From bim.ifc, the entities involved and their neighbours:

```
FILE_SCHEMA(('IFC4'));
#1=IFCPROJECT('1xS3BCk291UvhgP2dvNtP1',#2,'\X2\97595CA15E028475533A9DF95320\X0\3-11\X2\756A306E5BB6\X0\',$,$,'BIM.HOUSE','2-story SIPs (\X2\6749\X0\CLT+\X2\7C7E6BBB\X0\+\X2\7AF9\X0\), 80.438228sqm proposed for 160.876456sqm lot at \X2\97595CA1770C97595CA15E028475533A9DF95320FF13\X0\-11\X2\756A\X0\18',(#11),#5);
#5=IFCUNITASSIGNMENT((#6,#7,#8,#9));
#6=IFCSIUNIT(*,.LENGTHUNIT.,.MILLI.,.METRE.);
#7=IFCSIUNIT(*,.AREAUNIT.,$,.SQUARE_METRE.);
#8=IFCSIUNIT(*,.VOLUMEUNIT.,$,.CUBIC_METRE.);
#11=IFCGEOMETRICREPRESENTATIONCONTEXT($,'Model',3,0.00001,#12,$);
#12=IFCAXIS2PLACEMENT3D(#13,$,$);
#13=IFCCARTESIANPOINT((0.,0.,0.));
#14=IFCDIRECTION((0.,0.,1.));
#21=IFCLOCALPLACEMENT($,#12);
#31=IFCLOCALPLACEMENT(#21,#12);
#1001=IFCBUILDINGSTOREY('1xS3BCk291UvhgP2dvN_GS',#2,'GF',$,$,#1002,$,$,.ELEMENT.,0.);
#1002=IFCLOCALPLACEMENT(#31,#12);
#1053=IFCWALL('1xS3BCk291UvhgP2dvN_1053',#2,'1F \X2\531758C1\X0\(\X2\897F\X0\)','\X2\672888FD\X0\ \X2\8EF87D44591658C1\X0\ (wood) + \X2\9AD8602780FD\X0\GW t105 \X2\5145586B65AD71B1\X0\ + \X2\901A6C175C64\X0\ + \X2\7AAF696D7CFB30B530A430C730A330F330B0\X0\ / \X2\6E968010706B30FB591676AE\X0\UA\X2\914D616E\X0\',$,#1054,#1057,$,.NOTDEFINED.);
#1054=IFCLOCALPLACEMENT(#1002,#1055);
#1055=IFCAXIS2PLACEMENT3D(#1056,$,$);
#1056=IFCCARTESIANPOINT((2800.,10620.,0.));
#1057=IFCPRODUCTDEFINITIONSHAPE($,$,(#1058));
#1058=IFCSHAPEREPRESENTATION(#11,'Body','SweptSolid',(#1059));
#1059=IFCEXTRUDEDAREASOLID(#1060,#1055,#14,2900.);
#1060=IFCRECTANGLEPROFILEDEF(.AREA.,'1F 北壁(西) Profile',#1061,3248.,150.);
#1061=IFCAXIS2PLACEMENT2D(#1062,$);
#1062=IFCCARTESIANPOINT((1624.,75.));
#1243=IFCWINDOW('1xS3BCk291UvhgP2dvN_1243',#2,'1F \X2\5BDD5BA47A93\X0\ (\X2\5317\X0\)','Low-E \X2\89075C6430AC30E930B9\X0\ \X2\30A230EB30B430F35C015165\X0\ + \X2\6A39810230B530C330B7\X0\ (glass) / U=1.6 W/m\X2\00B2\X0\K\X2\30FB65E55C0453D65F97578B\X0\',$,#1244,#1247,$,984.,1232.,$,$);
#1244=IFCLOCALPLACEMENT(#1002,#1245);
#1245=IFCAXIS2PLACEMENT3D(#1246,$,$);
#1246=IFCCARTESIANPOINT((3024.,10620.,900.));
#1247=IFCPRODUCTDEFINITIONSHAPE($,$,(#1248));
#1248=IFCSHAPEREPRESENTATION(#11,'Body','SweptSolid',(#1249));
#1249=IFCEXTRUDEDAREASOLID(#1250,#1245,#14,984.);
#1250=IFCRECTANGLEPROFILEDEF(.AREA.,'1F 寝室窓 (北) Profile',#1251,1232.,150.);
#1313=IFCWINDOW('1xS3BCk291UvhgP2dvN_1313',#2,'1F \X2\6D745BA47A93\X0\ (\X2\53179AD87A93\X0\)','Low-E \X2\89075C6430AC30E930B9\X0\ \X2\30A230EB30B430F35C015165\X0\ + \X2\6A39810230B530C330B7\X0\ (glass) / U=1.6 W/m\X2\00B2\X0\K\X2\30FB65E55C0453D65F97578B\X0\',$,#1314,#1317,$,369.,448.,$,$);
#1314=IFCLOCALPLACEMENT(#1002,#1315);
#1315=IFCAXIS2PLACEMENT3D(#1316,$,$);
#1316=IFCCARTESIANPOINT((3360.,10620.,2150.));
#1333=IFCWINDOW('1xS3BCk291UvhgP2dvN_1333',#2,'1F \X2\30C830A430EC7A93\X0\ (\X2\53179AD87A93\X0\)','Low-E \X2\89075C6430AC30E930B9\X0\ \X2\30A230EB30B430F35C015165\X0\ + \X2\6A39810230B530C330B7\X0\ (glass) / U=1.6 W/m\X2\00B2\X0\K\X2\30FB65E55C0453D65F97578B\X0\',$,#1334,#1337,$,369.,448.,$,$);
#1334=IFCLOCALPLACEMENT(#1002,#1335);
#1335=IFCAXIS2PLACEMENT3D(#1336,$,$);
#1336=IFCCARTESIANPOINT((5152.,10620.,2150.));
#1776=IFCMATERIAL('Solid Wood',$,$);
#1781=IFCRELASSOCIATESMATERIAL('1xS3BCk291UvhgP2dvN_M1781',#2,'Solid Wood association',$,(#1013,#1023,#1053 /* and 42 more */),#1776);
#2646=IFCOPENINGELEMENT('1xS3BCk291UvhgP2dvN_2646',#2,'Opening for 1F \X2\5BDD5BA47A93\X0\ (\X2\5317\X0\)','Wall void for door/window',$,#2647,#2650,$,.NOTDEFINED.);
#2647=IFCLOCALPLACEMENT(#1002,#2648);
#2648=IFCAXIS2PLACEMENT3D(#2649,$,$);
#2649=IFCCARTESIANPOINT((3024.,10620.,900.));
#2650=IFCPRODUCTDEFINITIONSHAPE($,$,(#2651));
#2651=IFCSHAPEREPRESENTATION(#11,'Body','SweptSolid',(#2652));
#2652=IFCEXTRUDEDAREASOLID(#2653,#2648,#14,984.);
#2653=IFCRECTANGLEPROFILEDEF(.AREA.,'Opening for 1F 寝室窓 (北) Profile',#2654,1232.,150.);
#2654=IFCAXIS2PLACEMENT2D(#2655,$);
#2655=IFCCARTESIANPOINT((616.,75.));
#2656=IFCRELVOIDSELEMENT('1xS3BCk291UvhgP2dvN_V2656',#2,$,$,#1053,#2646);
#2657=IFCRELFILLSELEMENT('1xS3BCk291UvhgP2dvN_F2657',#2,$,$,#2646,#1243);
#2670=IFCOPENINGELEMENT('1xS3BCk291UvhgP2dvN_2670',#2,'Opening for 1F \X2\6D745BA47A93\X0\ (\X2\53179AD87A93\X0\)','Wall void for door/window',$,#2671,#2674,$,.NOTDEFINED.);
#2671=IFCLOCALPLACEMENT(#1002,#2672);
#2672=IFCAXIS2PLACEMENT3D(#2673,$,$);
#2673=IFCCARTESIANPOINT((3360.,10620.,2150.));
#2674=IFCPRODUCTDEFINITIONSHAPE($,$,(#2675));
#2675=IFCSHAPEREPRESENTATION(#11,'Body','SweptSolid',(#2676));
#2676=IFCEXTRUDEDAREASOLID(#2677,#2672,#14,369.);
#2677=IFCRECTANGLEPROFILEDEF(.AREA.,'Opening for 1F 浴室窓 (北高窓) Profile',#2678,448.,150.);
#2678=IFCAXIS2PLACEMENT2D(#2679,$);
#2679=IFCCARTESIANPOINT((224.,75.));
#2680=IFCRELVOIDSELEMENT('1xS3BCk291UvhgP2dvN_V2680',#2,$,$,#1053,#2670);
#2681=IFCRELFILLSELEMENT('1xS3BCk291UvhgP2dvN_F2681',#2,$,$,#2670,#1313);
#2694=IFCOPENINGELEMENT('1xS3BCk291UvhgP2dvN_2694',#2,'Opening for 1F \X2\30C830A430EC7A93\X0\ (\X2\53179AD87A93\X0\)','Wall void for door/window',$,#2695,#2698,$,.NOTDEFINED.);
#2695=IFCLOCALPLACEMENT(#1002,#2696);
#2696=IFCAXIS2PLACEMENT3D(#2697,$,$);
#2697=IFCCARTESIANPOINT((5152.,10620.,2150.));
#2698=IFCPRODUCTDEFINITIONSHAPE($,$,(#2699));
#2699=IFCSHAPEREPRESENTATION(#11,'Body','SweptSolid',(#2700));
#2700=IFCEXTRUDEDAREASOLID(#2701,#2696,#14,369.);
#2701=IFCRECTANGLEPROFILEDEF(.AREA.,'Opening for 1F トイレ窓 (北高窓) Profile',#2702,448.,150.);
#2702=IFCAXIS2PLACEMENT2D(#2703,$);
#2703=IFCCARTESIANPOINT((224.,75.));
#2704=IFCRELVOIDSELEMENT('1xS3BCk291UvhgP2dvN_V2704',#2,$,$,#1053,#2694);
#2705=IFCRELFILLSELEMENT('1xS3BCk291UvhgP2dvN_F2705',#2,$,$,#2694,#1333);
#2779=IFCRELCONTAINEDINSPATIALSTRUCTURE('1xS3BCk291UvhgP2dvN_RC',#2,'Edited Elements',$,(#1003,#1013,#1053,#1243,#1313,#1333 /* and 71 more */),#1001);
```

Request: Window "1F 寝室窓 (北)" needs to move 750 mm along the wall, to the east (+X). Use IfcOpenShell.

```python
import ifcopenshell
import ifcopenshell.api.geometry
import ifcopenshell.util.placement
import ifcopenshell.util.unit

model = ifcopenshell.open("bim.ifc")
unit_scale = ifcopenshell.util.unit.calculate_unit_scale(model)

window = model.by_id(1243)
opening = window.FillsVoids[0].RelatingOpeningElement
wall = opening.VoidsElements[0].RelatingBuildingElement

wall_matrix = ifcopenshell.util.placement.get_local_placement(wall.ObjectPlacement)
shift = wall_matrix[:3, 0] * 0.75 / unit_scale
before = ifcopenshell.util.placement.get_local_placement(window.ObjectPlacement)[:3, 3].copy()

# The window is not placed relative to its opening, so move both.
for product in (opening, window):
    matrix = ifcopenshell.util.placement.get_local_placement(product.ObjectPlacement)
    matrix[:3, 3] += shift
    ifcopenshell.api.geometry.edit_object_placement(model, product=product, matrix=matrix, is_si=False)

after = ifcopenshell.util.placement.get_local_placement(window.ObjectPlacement)[:3, 3]
print("window moved by", (after - before).round(3) + 0.0)

model.write("bim-out.ifc")
```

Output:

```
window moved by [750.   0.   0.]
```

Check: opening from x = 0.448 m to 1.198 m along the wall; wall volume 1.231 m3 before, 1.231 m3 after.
